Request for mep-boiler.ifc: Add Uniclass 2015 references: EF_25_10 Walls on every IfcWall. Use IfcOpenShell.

First a look at what the model holds.

```python
import ifcopenshell

model = ifcopenshell.open("mep-boiler.ifc")
print(model.schema)
print("classifications:", [c.Name for c in model.by_type("IfcClassification")])
for ifc_class in ("IfcDoor", "IfcRoof", "IfcStair", "IfcWall", "IfcWindow"):
    print(ifc_class, len(model.by_type(ifc_class)))
```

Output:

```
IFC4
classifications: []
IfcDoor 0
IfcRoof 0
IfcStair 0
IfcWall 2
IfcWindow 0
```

```python
import ifcopenshell
import ifcopenshell.api.classification

model = ifcopenshell.open("mep-boiler.ifc")

system = ifcopenshell.api.classification.add_classification(model, classification="Uniclass 2015")

codes = {
    "IfcWall": ("EF_25_10", "Walls"),
}
for ifc_class, (code, name) in codes.items():
    products = model.by_type(ifc_class)
    ifcopenshell.api.classification.add_reference(
        model, products=products, classification=system, identification=code, name=name
    )
    print(code, len(products))

model.write("mep-boiler-out.ifc")
```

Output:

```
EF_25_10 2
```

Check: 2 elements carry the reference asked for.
